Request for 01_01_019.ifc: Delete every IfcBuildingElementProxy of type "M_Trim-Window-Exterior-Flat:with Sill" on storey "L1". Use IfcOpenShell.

First a look at what the model holds.

```python
import ifcopenshell
import ifcopenshell.util.element

model = ifcopenshell.open("01_01_019.ifc")
print(model.schema)
storey = next(s for s in model.by_type("IfcBuildingStorey") if s.Name == "L1")
proxies = [e for e in ifcopenshell.util.element.get_decomposition(storey) if e.is_a("IfcBuildingElementProxy")]
seen = {}
for e in proxies:
    element_type = ifcopenshell.util.element.get_type(e)
    name = element_type.Name if element_type not in (None, e) else None
    seen[name] = seen.get(name, 0) + 1
for name, count in sorted(seen.items(), key=str):
    print(count, "x", name)
```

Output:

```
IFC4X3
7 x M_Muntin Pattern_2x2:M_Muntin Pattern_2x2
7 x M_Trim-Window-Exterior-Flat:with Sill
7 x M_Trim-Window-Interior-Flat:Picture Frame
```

```python
import ifcopenshell
import ifcopenshell.api.root
import ifcopenshell.util.element

model = ifcopenshell.open("01_01_019.ifc")

storey = next(s for s in model.by_type("IfcBuildingStorey") if s.Name == "L1")
proxies = [e for e in ifcopenshell.util.element.get_decomposition(storey) if e.is_a("IfcBuildingElementProxy")]
targets = [e for e in proxies if (t := ifcopenshell.util.element.get_type(e)) not in (None, e) and t.Name == "M_Trim-Window-Exterior-Flat:with Sill"]

for e in targets:
    ifcopenshell.api.root.remove_product(model, product=e)
print(len(targets), "removed")

model.write("01_01_019_v2.ifc")
```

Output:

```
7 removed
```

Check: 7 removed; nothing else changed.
